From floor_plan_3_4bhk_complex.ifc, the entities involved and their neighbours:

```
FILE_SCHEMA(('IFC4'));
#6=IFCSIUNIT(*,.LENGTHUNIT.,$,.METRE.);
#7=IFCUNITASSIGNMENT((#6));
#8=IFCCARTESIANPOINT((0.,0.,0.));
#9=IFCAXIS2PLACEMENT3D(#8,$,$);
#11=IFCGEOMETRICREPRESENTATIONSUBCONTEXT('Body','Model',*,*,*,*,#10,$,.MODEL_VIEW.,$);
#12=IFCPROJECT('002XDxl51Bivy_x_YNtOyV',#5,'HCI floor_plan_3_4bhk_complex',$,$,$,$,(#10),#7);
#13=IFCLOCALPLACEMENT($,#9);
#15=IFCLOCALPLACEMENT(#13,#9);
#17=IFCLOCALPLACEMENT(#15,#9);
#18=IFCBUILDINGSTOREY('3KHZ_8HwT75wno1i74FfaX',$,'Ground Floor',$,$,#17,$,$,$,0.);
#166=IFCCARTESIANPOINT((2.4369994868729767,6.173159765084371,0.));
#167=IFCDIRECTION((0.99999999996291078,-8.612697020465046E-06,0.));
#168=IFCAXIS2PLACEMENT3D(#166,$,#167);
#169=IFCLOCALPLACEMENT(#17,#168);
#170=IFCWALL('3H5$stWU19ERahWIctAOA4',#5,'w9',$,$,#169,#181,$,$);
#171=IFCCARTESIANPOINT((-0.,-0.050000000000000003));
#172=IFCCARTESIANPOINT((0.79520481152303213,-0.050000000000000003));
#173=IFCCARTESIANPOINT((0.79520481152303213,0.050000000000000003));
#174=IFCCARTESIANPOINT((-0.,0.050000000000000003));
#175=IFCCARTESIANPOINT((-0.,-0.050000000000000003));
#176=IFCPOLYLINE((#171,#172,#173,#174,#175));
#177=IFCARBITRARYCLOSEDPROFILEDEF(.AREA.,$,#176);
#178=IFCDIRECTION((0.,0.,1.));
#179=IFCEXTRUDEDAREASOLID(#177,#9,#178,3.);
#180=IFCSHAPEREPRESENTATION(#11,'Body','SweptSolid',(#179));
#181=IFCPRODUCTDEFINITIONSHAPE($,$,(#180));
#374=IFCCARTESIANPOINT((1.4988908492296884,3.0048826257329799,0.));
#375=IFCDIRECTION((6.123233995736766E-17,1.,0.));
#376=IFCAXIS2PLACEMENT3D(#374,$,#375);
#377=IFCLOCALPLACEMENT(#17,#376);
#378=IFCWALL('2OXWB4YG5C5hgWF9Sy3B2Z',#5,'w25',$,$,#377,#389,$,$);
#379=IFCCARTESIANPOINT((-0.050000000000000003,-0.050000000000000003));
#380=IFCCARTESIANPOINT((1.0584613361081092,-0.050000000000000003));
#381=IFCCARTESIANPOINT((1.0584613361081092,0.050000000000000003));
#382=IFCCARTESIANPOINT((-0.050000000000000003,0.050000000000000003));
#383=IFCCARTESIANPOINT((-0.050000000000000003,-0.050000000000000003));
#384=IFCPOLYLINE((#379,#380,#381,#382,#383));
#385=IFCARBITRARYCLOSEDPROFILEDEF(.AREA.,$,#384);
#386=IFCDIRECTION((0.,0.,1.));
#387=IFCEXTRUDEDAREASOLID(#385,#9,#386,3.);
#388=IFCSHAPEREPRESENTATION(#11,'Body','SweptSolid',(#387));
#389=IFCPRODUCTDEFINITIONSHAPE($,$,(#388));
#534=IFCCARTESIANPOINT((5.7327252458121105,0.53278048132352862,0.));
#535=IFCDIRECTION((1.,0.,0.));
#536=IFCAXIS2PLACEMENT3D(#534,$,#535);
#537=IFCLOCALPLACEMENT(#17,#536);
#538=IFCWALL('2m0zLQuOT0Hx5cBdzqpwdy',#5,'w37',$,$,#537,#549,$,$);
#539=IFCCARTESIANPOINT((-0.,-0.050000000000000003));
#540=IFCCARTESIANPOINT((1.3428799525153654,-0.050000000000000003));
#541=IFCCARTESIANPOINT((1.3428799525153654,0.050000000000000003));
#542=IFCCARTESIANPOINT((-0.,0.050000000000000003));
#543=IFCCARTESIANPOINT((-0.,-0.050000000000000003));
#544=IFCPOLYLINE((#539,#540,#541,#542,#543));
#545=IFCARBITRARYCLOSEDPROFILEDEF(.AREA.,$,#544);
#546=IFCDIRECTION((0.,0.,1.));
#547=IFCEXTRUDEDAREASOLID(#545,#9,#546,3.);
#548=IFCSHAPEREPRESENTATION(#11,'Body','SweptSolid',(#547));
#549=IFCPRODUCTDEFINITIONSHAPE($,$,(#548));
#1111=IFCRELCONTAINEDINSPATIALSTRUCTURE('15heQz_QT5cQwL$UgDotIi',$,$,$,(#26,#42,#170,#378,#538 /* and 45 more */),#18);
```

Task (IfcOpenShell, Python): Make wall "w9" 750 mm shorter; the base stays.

```python
import ifcopenshell
import ifcopenshell.geom
import ifcopenshell.util.representation
import ifcopenshell.util.shape
import ifcopenshell.util.unit

model = ifcopenshell.open("floor_plan_3_4bhk_complex.ifc")
unit_scale = ifcopenshell.util.unit.calculate_unit_scale(model)
settings = ifcopenshell.geom.settings()


def volume(element):
    """Net volume in cubic metres, openings subtracted."""
    shape = ifcopenshell.geom.create_shape(settings, element)
    return ifcopenshell.util.shape.get_volume(shape.geometry)


wall = model.by_guid("3H5$stWU19ERahWIctAOA4")
before = volume(wall)

body = ifcopenshell.util.representation.get_representation(wall, "Model", "Body")
solid = body.Items[0]
old_height = solid.Depth
solid.Depth -= 0.75 / unit_scale
after = volume(wall)

print(f"height {old_height:g} -> {solid.Depth:g}, volume {before:.3f} -> {after:.3f} m3")

model.write("floor_plan_3_4bhk_complex_v2.ifc")
```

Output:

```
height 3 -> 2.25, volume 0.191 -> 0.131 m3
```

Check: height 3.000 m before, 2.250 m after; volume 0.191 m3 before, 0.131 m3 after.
